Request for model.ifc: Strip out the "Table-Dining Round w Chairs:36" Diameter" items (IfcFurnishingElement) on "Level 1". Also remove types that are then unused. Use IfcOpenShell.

First a look at what the model holds.

```python
import ifcopenshell
import ifcopenshell.util.element

model = ifcopenshell.open("model.ifc")
print(model.schema)
storey = next(s for s in model.by_type("IfcBuildingStorey") if s.Name == "Level 1")
furniture = [e for e in ifcopenshell.util.element.get_decomposition(storey) if e.is_a("IfcFurnishingElement")]
seen = {}
for e in furniture:
    element_type = ifcopenshell.util.element.get_type(e)
    name = element_type.Name if element_type not in (None, e) else None
    seen[name] = seen.get(name, 0) + 1
for name, count in sorted(seen.items(), key=str):
    print(count, "x", name)
```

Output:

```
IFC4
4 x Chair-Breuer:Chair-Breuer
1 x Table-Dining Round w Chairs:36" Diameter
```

```python
import ifcopenshell
import ifcopenshell.api.root
import ifcopenshell.util.element

model = ifcopenshell.open("model.ifc")

storey = next(s for s in model.by_type("IfcBuildingStorey") if s.Name == "Level 1")
furniture = [e for e in ifcopenshell.util.element.get_decomposition(storey) if e.is_a("IfcFurnishingElement")]
targets = [e for e in furniture if (t := ifcopenshell.util.element.get_type(e)) not in (None, e) and t.Name == 'Table-Dining Round w Chairs:36" Diameter']
types = {ifcopenshell.util.element.get_type(e) for e in targets} - {None, *targets}

for e in targets:
    ifcopenshell.api.root.remove_product(model, product=e)
print(len(targets), "removed")

unused = [t for t in types if not ifcopenshell.util.element.get_types(t)]
for t in unused:
    ifcopenshell.api.root.remove_product(model, product=t)
print(len(unused), "unused types removed")

model.write("model_v2.ifc")
```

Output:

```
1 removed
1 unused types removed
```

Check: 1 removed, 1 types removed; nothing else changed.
